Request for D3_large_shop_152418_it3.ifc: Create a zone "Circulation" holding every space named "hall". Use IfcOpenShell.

First a look at what the model holds.

```python
import ifcopenshell

model = ifcopenshell.open("D3_large_shop_152418_it3.ifc")
print(model.schema)
seen = {}
for space in model.by_type("IfcSpace"):
    seen[space.LongName] = seen.get(space.LongName, 0) + 1
for name, count in sorted(seen.items(), key=str):
    print(count, "x", name)
print("zones:", [z.Name for z in model.by_type("IfcZone")][:20])
```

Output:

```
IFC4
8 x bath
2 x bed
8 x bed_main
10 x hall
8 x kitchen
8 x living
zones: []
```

```python
import ifcopenshell
import ifcopenshell.api.group
import ifcopenshell.api.root

model = ifcopenshell.open("D3_large_shop_152418_it3.ifc")

names = {"hall"}
spaces = [s for s in model.by_type("IfcSpace") if s.LongName in names]

zone = ifcopenshell.api.root.create_entity(model, ifc_class="IfcZone", name="Circulation")
ifcopenshell.api.group.assign_group(model, products=spaces, group=zone)
print(len(spaces), "spaces in", zone.Name)

model.write("D3_large_shop_152418_it3_rev.ifc")
```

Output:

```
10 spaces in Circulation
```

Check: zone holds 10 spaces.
